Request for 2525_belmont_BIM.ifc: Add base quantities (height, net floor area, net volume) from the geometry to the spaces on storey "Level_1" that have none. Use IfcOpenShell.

First a look at what the model holds.

```python
import ifcopenshell
import ifcopenshell.util.element
import ifcopenshell.util.unit

model = ifcopenshell.open("2525_belmont_BIM.ifc")
print(model.schema)
for unit_type in ("LENGTHUNIT", "AREAUNIT", "VOLUMEUNIT"):
    print(unit_type, ifcopenshell.util.unit.calculate_unit_scale(model, unit_type))
storey = next(s for s in model.by_type("IfcBuildingStorey") if s.Name == "Level_1")
spaces = [e for e in ifcopenshell.util.element.get_decomposition(storey) if e.is_a("IfcSpace")]
for e in sorted(spaces, key=lambda e: e.id()):
    print(e.id(), e.is_a(), e.Name, list(ifcopenshell.util.element.get_psets(e, qtos_only=True)), sep=" | ")
```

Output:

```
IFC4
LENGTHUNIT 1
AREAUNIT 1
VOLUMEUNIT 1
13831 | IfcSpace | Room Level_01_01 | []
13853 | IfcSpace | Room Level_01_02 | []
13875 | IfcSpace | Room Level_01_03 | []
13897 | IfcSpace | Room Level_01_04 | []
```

```python
import ifcopenshell
import ifcopenshell.api.pset
import ifcopenshell.geom
import ifcopenshell.util.element
import ifcopenshell.util.shape
import ifcopenshell.util.unit

model = ifcopenshell.open("2525_belmont_BIM.ifc")
unit_scale = ifcopenshell.util.unit.calculate_unit_scale(model)
area_scale = ifcopenshell.util.unit.calculate_unit_scale(model, "AREAUNIT")
volume_scale = ifcopenshell.util.unit.calculate_unit_scale(model, "VOLUMEUNIT")
settings = ifcopenshell.geom.settings()

storey = next(s for s in model.by_type("IfcBuildingStorey") if s.Name == "Level_1")
spaces = [e for e in ifcopenshell.util.element.get_decomposition(storey) if e.is_a("IfcSpace")]

for e in sorted(spaces, key=lambda e: e.id()):
    if ifcopenshell.util.element.get_psets(e, qtos_only=True, should_inherit=False):
        continue
    # Geometry comes back in metres, in the element's own axes.
    shape = ifcopenshell.geom.create_shape(settings, e)
    values = {
        "Height": ifcopenshell.util.shape.get_z(shape.geometry) / unit_scale,
        "NetFloorArea": ifcopenshell.util.shape.get_footprint_area(shape.geometry) / area_scale,
        "NetVolume": ifcopenshell.util.shape.get_volume(shape.geometry) / volume_scale,
    }
    qto = ifcopenshell.api.pset.add_qto(model, product=e, name="Qto_SpaceBaseQuantities")
    ifcopenshell.api.pset.edit_qto(model, qto=qto, properties=values)
    print(e.id(), {k: round(v, 3) for k, v in values.items()})

model.write("2525_belmont_BIM_v2.ifc")
```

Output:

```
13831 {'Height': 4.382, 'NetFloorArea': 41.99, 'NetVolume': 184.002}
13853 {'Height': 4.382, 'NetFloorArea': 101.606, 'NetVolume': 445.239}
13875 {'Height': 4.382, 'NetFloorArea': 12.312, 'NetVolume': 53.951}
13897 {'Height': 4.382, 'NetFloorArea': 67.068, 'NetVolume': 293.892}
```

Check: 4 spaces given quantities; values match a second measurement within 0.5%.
